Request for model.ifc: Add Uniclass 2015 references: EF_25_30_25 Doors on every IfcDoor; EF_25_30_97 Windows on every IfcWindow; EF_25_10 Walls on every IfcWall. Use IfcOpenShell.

First a look at what the model holds.

```python
import ifcopenshell

model = ifcopenshell.open("model.ifc")
print(model.schema)
print("classifications:", [c.Name for c in model.by_type("IfcClassification")])
for ifc_class in ("IfcDoor", "IfcRoof", "IfcStair", "IfcWall", "IfcWindow"):
    print(ifc_class, len(model.by_type(ifc_class)))
```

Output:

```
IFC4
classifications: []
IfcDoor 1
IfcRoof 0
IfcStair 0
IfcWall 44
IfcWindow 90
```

```python
import ifcopenshell
import ifcopenshell.api.classification

model = ifcopenshell.open("model.ifc")

system = ifcopenshell.api.classification.add_classification(model, classification="Uniclass 2015")

codes = {
    "IfcDoor": ("EF_25_30_25", "Doors"),
    "IfcWindow": ("EF_25_30_97", "Windows"),
    "IfcWall": ("EF_25_10", "Walls"),
}
for ifc_class, (code, name) in codes.items():
    products = model.by_type(ifc_class)
    ifcopenshell.api.classification.add_reference(
        model, products=products, classification=system, identification=code, name=name
    )
    print(code, len(products))

model.write("model_rev.ifc")
```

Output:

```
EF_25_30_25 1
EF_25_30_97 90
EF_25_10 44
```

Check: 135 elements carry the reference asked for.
